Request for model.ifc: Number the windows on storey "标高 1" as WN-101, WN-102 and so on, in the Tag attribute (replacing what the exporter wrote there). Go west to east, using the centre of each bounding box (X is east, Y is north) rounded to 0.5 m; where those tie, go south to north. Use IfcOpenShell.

First a look at what the model holds.

```python
import ifcopenshell
import ifcopenshell.util.element
import ifcopenshell.util.placement

model = ifcopenshell.open("model.ifc")
print(model.schema)
storey = next(s for s in model.by_type("IfcBuildingStorey") if s.Name == "标高 1")
windows = [e for e in ifcopenshell.util.element.get_decomposition(storey) if e.is_a("IfcWindow")]
for e in sorted(windows, key=lambda e: e.id()):
    origin = ifcopenshell.util.placement.get_local_placement(e.ObjectPlacement)[:3, 3]
    print(e.id(), e.Tag, e.Name, origin.round(2) + 0.0, sep=" | ")
```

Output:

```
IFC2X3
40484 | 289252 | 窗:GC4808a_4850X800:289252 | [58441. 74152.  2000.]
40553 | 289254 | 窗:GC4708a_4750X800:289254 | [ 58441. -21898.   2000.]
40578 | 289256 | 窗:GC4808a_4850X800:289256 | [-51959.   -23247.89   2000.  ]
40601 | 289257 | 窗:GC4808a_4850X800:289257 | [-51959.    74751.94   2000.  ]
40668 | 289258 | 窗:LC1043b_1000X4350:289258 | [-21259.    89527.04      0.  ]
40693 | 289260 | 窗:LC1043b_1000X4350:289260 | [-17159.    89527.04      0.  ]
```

```python
import ifcopenshell
import ifcopenshell.geom
import ifcopenshell.util.element
import ifcopenshell.util.shape

model = ifcopenshell.open("model.ifc")
settings = ifcopenshell.geom.settings()
settings.set("use-world-coords", True)


def centre(element):
    shape = ifcopenshell.geom.create_shape(settings, element)
    return ifcopenshell.util.shape.get_bbox_centroid(shape.geometry)


storey = next(s for s in model.by_type("IfcBuildingStorey") if s.Name == "标高 1")
windows = [e for e in ifcopenshell.util.element.get_decomposition(storey) if e.is_a("IfcWindow")]

# Insertion points can sit at a corner or the storey origin, so sort by the geometry (in metres).
centres = {e: centre(e) for e in windows}
windows.sort(key=lambda e: (round(centres[e][0] / 0.5), centres[e][1]))

for i, e in enumerate(windows, start=1):
    number = f"WN-1{i:02d}"
    e.Tag = number
    print(e.id(), number)

model.write("model_edited.ifc")
```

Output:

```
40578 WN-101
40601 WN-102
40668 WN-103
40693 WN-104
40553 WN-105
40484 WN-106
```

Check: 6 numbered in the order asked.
